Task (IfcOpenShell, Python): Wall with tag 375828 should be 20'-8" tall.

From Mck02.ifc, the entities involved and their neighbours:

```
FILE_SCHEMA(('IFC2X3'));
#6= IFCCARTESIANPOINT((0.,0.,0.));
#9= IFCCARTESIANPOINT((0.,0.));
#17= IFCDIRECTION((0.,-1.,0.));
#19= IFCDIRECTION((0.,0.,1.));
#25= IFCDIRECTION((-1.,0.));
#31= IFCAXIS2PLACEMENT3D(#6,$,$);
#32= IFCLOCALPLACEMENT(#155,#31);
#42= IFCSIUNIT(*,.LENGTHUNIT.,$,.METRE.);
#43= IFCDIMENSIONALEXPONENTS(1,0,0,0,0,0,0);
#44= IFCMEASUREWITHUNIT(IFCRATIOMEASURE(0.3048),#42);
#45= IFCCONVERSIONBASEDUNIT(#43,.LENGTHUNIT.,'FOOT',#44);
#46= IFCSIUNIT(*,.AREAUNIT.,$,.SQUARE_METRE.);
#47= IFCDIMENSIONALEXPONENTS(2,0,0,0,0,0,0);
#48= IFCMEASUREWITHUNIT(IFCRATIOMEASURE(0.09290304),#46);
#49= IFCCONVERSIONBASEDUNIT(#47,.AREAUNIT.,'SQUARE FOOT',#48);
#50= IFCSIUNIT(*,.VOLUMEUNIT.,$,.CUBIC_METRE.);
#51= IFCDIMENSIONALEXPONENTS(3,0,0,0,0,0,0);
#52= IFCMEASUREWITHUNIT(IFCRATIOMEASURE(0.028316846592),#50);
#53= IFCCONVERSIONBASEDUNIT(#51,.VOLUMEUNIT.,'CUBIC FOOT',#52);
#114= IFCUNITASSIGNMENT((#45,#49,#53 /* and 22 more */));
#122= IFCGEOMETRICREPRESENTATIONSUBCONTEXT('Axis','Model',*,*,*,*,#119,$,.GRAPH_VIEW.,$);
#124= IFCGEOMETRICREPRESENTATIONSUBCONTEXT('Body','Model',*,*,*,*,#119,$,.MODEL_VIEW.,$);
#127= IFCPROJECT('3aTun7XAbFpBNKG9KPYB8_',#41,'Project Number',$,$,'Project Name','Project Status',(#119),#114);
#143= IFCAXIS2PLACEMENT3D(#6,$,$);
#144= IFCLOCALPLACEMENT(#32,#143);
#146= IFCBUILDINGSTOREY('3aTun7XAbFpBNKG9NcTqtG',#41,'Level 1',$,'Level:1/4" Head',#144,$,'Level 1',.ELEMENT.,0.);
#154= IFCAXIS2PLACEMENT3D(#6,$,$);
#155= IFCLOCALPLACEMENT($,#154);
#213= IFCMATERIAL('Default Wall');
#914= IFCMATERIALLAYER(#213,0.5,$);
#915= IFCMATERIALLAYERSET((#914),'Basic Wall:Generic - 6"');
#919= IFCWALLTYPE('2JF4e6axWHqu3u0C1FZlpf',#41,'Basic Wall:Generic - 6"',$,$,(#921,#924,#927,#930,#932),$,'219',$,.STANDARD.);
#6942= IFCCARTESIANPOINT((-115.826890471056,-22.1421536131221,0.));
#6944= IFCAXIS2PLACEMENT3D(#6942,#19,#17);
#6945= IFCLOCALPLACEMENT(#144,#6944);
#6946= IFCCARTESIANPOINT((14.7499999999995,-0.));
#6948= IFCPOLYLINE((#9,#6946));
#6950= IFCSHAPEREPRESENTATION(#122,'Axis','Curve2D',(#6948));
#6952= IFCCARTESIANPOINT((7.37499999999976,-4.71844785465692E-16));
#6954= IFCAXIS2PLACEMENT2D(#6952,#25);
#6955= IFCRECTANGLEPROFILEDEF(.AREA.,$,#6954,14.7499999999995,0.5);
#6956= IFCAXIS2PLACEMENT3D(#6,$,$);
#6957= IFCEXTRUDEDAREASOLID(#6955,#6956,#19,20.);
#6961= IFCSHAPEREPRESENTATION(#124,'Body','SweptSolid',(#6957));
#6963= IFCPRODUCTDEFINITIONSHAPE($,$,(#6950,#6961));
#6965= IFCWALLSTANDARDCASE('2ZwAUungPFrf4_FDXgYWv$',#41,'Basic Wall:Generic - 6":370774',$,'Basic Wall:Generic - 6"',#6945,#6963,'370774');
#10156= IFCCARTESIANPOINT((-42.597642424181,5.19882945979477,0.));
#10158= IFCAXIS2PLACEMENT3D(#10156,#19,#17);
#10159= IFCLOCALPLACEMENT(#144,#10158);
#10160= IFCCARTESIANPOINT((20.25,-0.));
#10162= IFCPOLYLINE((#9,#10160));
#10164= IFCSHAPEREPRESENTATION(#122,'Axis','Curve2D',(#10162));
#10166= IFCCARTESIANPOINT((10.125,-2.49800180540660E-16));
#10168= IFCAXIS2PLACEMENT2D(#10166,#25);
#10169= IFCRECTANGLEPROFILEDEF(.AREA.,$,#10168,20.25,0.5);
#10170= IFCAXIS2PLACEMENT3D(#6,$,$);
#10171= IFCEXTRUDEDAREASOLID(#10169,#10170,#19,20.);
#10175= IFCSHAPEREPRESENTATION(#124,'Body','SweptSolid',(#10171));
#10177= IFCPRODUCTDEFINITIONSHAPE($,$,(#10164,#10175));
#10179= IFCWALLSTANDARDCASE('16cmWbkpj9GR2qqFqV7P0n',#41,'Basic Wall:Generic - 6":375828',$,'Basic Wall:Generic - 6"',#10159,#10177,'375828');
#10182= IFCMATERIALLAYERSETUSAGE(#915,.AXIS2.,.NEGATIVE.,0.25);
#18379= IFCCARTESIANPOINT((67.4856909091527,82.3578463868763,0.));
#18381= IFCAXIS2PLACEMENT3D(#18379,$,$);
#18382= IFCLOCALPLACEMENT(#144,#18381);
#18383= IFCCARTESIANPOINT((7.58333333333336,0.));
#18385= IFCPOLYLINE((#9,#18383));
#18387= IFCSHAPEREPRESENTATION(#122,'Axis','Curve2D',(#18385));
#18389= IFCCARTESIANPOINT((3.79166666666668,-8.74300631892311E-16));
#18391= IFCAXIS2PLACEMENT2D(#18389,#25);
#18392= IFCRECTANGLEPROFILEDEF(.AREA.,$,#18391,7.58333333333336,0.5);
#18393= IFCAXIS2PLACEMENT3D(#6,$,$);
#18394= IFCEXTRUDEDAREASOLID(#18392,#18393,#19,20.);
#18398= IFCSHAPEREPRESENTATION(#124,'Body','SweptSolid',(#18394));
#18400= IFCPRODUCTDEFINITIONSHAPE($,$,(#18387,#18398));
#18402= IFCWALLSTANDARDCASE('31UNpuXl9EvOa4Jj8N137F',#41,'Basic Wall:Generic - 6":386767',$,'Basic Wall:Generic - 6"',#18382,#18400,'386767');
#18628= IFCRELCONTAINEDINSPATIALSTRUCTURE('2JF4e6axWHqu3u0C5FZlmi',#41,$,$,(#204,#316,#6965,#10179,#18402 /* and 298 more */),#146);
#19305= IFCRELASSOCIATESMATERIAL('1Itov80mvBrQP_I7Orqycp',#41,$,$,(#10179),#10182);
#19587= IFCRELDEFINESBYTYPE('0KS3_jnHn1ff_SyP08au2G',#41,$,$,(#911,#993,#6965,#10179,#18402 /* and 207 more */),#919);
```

```python
import ifcopenshell
import ifcopenshell.geom
import ifcopenshell.util.representation
import ifcopenshell.util.shape
import ifcopenshell.util.unit

model = ifcopenshell.open("Mck02.ifc")
unit_scale = ifcopenshell.util.unit.calculate_unit_scale(model)
settings = ifcopenshell.geom.settings()


def volume(element):
    """Net volume in cubic metres, openings subtracted."""
    shape = ifcopenshell.geom.create_shape(settings, element)
    return ifcopenshell.util.shape.get_volume(shape.geometry)


wall = model.by_guid("16cmWbkpj9GR2qqFqV7P0n")
before = volume(wall)

body = ifcopenshell.util.representation.get_representation(wall, "Model", "Body")
solid = body.Items[0]
old_height = solid.Depth
solid.Depth = 248 * 0.0254 / unit_scale
after = volume(wall)

print(f"height {old_height:g} -> {solid.Depth:g}, volume {before:.3f} -> {after:.3f} m3")

model.write("Mck02_edited.ifc")
```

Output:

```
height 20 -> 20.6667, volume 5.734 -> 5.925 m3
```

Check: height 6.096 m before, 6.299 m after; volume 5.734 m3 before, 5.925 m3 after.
